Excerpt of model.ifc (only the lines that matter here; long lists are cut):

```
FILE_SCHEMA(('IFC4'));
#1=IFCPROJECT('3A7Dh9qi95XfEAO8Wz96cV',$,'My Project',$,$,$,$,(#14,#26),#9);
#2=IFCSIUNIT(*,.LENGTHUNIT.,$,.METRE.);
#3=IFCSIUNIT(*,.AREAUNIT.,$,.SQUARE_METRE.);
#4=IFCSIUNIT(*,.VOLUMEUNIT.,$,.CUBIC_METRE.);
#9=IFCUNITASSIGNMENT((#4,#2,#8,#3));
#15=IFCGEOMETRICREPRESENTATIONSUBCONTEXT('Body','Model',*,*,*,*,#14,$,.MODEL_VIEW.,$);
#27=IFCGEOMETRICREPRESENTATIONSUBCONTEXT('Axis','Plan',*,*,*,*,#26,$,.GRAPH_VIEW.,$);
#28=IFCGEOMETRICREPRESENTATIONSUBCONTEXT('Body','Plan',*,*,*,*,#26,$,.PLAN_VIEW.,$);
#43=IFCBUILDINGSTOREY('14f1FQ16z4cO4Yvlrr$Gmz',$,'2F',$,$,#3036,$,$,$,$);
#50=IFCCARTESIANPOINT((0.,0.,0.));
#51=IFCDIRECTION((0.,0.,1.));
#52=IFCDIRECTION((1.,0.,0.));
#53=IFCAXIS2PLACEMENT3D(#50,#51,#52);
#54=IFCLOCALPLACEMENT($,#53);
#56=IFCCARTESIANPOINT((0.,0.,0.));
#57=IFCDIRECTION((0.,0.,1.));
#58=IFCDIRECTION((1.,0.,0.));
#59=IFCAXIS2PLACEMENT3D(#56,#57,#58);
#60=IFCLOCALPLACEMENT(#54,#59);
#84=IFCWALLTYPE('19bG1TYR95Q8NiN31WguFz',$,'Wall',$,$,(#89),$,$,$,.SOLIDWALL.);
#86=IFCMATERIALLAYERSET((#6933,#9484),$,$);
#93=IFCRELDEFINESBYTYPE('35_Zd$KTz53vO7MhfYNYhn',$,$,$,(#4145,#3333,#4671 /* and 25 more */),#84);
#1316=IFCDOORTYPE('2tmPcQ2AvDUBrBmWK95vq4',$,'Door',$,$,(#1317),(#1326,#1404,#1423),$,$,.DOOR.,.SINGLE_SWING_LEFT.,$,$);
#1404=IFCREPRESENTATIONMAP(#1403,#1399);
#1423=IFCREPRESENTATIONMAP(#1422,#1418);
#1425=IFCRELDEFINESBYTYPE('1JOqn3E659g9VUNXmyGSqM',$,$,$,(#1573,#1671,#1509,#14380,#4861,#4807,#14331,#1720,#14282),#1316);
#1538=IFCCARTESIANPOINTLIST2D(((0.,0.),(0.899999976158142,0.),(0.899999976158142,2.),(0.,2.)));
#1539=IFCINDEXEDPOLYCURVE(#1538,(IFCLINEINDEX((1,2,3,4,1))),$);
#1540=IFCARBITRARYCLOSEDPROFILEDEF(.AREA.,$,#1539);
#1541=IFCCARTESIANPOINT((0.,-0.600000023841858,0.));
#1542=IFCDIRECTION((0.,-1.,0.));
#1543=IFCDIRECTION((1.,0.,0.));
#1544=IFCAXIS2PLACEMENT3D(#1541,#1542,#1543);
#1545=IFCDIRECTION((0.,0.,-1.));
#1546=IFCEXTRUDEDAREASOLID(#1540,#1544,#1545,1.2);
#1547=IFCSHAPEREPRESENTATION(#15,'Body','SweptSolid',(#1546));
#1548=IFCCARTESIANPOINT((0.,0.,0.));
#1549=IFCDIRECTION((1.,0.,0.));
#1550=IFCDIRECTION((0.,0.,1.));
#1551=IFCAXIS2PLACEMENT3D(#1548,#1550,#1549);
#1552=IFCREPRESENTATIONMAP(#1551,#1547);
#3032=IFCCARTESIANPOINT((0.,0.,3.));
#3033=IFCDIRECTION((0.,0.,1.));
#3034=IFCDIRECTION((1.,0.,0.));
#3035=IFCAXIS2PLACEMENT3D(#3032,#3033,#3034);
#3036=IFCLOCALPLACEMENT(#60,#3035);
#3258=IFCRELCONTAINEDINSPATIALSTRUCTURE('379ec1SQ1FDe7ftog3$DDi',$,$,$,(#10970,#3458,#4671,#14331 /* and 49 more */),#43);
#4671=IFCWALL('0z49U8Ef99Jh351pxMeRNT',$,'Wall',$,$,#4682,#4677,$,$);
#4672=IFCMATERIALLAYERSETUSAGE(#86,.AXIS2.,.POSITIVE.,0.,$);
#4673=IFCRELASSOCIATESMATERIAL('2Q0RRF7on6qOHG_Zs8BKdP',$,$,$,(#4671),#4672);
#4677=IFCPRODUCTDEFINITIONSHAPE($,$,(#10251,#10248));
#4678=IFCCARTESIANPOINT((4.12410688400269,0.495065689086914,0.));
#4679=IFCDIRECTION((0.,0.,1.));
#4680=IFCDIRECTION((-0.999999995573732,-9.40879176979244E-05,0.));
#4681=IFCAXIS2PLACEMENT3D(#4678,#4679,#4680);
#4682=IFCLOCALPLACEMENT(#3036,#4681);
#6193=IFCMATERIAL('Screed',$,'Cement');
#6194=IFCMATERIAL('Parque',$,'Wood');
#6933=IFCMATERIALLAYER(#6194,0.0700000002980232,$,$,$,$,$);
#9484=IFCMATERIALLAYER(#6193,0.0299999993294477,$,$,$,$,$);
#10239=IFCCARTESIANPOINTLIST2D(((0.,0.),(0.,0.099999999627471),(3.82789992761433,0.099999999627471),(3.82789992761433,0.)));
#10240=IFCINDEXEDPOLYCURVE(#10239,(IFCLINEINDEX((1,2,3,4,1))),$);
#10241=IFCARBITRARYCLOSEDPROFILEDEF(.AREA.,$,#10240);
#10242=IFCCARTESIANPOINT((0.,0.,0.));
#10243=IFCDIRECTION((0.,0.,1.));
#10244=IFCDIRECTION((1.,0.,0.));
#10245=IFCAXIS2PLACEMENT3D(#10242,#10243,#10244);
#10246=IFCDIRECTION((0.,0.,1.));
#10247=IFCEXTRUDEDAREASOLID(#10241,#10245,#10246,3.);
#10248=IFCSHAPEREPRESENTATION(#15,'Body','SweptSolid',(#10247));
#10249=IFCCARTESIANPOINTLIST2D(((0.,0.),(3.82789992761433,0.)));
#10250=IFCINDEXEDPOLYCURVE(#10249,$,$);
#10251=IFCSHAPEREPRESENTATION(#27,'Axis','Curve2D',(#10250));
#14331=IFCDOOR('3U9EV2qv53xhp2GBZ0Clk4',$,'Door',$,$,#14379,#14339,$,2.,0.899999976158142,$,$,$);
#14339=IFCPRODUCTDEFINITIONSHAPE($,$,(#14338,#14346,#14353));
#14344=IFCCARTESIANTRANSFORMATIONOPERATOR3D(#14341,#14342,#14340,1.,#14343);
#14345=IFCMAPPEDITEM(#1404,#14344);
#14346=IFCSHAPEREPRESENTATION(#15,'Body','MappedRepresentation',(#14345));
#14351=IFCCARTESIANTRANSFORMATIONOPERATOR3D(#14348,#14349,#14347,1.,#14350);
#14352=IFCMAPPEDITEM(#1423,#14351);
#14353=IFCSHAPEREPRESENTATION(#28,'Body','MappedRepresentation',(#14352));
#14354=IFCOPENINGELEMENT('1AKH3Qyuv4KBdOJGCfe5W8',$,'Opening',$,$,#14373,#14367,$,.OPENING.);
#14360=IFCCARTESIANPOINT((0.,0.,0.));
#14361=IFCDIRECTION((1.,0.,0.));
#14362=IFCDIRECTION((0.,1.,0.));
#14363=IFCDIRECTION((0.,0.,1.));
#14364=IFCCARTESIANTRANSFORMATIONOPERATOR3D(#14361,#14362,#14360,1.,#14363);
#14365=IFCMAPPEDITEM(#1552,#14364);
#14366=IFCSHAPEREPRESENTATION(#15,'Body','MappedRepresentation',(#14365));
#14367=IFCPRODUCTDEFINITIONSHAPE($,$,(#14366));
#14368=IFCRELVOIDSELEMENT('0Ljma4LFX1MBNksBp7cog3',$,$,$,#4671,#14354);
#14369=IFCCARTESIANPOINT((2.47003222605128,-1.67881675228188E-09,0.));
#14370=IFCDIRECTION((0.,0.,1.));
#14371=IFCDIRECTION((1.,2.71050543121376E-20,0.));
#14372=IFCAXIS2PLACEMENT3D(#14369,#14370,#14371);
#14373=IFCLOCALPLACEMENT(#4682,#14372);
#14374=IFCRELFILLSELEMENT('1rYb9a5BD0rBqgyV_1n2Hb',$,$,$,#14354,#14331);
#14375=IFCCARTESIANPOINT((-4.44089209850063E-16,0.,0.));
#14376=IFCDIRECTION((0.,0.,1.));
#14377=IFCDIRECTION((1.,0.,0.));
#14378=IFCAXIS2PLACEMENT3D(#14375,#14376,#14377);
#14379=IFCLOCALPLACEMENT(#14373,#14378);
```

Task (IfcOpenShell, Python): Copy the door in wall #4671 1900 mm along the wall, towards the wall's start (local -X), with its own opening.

```python
import ifcopenshell
import ifcopenshell.api.feature
import ifcopenshell.api.geometry
import ifcopenshell.api.root
import ifcopenshell.geom
import ifcopenshell.util.element
import ifcopenshell.util.placement
import ifcopenshell.util.shape
import ifcopenshell.util.unit

model = ifcopenshell.open("model.ifc")
unit_scale = ifcopenshell.util.unit.calculate_unit_scale(model)
settings = ifcopenshell.geom.settings()


def volume(element):
    """Net volume in cubic metres, openings subtracted."""
    shape = ifcopenshell.geom.create_shape(settings, element)
    return ifcopenshell.util.shape.get_volume(shape.geometry)


door = model.by_guid("3U9EV2qv53xhp2GBZ0Clk4")
opening = door.FillsVoids[0].RelatingOpeningElement
wall = opening.VoidsElements[0].RelatingBuildingElement
before = volume(wall)
shift = ifcopenshell.util.placement.get_local_placement(wall.ObjectPlacement)[:3, 0] * -1.9 / unit_scale

# copy_class copies the void relationship, type, container and properties, but no geometry.
new_opening = ifcopenshell.api.root.copy_class(model, product=opening)
new_opening.Representation = ifcopenshell.util.element.copy_deep(
    model, opening.Representation, exclude=["IfcGeometricRepresentationContext", "IfcRepresentationMap"]
)
new_door = ifcopenshell.api.root.copy_class(model, product=door)
new_door.Representation = ifcopenshell.util.element.copy_deep(
    model, door.Representation, exclude=["IfcGeometricRepresentationContext", "IfcRepresentationMap"]
)
ifcopenshell.api.feature.add_filling(model, opening=new_opening, element=new_door)

for old, new in ((opening, new_opening), (door, new_door)):
    matrix = ifcopenshell.util.placement.get_local_placement(old.ObjectPlacement)
    matrix[:3, 3] += shift
    ifcopenshell.api.geometry.edit_object_placement(model, product=new, matrix=matrix, is_si=False)

after = volume(wall)

print(f"wall volume {before:.3f} -> {after:.3f} m3")

model.write("model_edited.ifc")
```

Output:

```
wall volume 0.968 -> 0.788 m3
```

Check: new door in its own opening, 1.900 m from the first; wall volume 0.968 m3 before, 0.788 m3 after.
